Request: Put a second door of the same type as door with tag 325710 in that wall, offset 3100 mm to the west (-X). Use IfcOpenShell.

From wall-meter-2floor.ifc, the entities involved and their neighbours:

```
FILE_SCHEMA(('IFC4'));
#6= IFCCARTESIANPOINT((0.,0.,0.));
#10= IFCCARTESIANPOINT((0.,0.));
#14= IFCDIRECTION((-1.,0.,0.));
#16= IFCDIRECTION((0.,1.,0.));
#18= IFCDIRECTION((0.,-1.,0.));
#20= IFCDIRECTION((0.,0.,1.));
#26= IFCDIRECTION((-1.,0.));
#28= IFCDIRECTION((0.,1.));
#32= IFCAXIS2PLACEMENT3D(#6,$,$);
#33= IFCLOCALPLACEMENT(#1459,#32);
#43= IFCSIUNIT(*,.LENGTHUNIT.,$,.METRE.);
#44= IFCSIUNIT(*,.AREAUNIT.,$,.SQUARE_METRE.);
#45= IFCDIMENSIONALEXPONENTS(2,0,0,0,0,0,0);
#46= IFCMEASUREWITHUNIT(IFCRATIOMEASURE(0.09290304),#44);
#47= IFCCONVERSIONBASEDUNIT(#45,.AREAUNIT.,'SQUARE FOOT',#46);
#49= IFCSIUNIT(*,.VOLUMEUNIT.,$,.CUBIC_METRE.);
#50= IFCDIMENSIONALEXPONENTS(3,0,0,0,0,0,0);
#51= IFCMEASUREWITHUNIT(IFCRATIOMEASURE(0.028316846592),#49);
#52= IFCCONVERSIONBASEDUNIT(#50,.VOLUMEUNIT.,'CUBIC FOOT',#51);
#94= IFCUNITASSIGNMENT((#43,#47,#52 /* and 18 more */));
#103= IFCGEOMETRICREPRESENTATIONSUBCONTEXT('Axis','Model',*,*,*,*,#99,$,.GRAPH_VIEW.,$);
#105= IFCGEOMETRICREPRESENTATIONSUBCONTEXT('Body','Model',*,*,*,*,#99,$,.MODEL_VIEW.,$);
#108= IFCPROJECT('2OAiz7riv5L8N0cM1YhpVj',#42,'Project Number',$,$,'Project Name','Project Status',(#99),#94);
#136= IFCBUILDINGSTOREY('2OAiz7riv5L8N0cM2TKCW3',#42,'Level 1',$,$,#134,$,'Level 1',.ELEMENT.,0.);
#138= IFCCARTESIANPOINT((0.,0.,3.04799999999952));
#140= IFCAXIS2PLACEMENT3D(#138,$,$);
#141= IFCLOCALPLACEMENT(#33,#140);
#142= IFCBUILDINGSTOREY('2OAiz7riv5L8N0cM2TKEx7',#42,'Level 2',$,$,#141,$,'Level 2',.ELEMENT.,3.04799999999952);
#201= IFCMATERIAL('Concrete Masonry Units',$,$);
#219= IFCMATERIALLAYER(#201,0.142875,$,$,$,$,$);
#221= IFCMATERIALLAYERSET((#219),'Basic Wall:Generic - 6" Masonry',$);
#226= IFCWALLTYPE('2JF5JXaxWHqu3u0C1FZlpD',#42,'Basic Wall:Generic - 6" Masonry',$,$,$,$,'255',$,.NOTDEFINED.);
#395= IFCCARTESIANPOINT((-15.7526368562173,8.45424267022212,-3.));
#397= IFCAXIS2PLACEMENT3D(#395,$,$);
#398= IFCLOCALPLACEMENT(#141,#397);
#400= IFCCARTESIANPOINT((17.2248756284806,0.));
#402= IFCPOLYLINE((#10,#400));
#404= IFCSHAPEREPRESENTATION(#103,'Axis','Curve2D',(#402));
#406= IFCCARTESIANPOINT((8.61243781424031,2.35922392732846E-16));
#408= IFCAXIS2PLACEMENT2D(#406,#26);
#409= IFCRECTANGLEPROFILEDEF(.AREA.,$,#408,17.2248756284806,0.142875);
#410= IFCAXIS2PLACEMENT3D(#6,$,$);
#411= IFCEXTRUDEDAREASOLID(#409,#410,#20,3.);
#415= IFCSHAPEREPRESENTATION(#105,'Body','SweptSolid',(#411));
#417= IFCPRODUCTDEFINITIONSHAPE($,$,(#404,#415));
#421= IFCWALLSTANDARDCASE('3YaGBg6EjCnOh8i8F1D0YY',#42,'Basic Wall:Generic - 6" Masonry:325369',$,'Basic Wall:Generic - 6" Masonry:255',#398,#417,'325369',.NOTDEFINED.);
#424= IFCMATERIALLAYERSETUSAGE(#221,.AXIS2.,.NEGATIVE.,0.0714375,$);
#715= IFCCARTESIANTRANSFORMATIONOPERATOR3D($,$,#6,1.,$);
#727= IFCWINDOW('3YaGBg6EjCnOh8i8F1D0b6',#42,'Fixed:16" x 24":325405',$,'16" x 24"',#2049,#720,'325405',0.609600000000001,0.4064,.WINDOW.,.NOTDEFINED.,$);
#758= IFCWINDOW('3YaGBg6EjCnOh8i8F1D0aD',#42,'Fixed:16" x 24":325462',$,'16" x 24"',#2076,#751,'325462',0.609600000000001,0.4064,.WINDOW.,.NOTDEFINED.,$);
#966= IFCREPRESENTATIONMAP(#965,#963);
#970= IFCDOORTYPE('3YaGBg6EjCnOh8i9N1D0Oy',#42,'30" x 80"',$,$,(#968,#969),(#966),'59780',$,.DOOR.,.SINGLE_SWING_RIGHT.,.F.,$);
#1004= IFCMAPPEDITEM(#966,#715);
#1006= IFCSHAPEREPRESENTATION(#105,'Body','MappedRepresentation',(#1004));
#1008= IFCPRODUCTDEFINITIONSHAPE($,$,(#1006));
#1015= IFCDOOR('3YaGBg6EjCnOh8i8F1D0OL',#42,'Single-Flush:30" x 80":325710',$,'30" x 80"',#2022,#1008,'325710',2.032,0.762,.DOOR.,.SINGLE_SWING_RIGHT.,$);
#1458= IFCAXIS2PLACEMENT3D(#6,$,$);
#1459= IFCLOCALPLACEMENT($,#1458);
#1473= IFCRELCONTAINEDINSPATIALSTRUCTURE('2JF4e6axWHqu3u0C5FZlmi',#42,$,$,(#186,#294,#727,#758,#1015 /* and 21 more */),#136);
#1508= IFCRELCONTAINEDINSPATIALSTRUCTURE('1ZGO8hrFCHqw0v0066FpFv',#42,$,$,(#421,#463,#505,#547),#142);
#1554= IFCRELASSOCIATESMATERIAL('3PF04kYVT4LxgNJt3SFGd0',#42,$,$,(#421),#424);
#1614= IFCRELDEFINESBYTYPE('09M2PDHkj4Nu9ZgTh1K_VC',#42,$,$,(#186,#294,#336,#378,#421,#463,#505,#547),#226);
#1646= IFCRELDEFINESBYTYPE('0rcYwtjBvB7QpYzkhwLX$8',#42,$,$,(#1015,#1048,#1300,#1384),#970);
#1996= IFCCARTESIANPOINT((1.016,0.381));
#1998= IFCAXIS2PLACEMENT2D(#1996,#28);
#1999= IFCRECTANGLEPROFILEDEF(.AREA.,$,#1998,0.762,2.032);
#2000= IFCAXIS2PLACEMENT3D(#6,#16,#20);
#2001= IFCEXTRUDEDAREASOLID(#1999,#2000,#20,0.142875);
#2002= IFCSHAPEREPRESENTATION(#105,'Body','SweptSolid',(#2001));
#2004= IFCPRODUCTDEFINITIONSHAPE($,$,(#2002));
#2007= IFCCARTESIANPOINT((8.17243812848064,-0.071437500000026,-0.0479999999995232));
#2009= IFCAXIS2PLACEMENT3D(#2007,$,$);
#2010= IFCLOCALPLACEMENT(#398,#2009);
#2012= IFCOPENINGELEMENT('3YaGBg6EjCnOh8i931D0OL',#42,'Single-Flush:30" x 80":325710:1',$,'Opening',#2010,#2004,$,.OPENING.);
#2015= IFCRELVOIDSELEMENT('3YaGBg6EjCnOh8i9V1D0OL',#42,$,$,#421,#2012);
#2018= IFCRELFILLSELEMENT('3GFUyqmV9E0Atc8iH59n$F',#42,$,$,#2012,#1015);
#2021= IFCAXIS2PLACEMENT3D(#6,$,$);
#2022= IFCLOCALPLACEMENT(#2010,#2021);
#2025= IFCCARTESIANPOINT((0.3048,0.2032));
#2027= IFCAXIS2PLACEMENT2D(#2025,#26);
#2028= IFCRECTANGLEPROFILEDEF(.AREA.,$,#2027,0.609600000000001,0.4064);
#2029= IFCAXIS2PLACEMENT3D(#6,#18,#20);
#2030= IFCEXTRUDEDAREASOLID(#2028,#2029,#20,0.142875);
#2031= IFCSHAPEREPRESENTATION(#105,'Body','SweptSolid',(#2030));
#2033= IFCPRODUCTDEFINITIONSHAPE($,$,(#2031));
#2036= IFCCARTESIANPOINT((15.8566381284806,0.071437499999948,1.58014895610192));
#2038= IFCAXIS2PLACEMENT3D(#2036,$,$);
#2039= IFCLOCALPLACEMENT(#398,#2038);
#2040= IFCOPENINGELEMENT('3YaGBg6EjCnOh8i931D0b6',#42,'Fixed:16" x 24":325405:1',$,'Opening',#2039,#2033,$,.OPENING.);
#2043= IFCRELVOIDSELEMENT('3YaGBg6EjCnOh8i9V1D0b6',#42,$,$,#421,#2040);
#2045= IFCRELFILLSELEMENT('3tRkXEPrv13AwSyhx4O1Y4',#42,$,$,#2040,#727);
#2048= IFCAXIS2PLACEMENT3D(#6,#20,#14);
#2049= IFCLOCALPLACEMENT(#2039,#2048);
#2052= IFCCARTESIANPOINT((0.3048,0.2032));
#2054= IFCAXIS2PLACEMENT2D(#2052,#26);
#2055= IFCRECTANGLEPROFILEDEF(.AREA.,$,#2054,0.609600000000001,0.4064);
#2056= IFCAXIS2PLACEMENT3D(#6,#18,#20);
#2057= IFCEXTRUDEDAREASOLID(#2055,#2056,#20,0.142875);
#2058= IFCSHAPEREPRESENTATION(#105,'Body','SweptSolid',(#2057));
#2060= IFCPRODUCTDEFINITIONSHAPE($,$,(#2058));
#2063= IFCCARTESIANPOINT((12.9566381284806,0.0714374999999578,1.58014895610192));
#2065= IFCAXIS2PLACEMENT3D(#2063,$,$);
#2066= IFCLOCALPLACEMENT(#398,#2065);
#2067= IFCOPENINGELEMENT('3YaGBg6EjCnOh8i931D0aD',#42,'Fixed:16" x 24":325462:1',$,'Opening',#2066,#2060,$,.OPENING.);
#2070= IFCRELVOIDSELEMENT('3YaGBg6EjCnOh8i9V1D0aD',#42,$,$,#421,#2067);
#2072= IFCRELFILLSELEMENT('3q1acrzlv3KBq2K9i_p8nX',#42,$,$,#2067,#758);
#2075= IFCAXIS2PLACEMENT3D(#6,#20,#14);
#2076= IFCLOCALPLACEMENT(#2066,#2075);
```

```python
import ifcopenshell
import ifcopenshell.api.feature
import ifcopenshell.api.geometry
import ifcopenshell.api.root
import ifcopenshell.geom
import ifcopenshell.util.element
import ifcopenshell.util.placement
import ifcopenshell.util.shape
import ifcopenshell.util.unit

model = ifcopenshell.open("wall-meter-2floor.ifc")
unit_scale = ifcopenshell.util.unit.calculate_unit_scale(model)
settings = ifcopenshell.geom.settings()


def volume(element):
    """Net volume in cubic metres, openings subtracted."""
    shape = ifcopenshell.geom.create_shape(settings, element)
    return ifcopenshell.util.shape.get_volume(shape.geometry)


def reuse_history(source, copy):
    """copy_class also copies each property set's owner history, people and application; keep the originals."""
    for rel in copy.IsDefinedBy:
        if rel.is_a("IfcRelDefinesByProperties") and (history := rel.RelatingPropertyDefinition.OwnerHistory):
            rel.RelatingPropertyDefinition.OwnerHistory = source.OwnerHistory
            ifcopenshell.util.element.remove_deep2(model, history)


door = model.by_guid("3YaGBg6EjCnOh8i8F1D0OL")
opening = door.FillsVoids[0].RelatingOpeningElement
wall = opening.VoidsElements[0].RelatingBuildingElement
before = volume(wall)
shift = ifcopenshell.util.placement.get_local_placement(wall.ObjectPlacement)[:3, 0] * -3.1 / unit_scale

# copy_class copies the void relationship, type, container and properties, but no geometry.
new_opening = ifcopenshell.api.root.copy_class(model, product=opening)
new_opening.Representation = ifcopenshell.util.element.copy_deep(
    model, opening.Representation, exclude=["IfcGeometricRepresentationContext", "IfcRepresentationMap"]
)
new_opening.Name = 'Single-Flush:30" x 80"'
new_door = ifcopenshell.api.root.copy_class(model, product=door)
new_door.Representation = ifcopenshell.util.element.copy_deep(
    model, door.Representation, exclude=["IfcGeometricRepresentationContext", "IfcRepresentationMap"]
)
new_door.Name = 'Single-Flush:30" x 80"'
new_door.Tag = None
reuse_history(door, new_door)
ifcopenshell.api.feature.add_filling(model, opening=new_opening, element=new_door)

for old, new in ((opening, new_opening), (door, new_door)):
    matrix = ifcopenshell.util.placement.get_local_placement(old.ObjectPlacement)
    matrix[:3, 3] += shift
    ifcopenshell.api.geometry.edit_object_placement(model, product=new, matrix=matrix, is_si=False)

after = volume(wall)

print(f"wall volume {before:.3f} -> {after:.3f} m3")

model.write("wall-meter-2floor_updated.ifc")
```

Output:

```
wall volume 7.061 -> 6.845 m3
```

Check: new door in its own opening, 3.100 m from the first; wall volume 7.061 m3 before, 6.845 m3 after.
